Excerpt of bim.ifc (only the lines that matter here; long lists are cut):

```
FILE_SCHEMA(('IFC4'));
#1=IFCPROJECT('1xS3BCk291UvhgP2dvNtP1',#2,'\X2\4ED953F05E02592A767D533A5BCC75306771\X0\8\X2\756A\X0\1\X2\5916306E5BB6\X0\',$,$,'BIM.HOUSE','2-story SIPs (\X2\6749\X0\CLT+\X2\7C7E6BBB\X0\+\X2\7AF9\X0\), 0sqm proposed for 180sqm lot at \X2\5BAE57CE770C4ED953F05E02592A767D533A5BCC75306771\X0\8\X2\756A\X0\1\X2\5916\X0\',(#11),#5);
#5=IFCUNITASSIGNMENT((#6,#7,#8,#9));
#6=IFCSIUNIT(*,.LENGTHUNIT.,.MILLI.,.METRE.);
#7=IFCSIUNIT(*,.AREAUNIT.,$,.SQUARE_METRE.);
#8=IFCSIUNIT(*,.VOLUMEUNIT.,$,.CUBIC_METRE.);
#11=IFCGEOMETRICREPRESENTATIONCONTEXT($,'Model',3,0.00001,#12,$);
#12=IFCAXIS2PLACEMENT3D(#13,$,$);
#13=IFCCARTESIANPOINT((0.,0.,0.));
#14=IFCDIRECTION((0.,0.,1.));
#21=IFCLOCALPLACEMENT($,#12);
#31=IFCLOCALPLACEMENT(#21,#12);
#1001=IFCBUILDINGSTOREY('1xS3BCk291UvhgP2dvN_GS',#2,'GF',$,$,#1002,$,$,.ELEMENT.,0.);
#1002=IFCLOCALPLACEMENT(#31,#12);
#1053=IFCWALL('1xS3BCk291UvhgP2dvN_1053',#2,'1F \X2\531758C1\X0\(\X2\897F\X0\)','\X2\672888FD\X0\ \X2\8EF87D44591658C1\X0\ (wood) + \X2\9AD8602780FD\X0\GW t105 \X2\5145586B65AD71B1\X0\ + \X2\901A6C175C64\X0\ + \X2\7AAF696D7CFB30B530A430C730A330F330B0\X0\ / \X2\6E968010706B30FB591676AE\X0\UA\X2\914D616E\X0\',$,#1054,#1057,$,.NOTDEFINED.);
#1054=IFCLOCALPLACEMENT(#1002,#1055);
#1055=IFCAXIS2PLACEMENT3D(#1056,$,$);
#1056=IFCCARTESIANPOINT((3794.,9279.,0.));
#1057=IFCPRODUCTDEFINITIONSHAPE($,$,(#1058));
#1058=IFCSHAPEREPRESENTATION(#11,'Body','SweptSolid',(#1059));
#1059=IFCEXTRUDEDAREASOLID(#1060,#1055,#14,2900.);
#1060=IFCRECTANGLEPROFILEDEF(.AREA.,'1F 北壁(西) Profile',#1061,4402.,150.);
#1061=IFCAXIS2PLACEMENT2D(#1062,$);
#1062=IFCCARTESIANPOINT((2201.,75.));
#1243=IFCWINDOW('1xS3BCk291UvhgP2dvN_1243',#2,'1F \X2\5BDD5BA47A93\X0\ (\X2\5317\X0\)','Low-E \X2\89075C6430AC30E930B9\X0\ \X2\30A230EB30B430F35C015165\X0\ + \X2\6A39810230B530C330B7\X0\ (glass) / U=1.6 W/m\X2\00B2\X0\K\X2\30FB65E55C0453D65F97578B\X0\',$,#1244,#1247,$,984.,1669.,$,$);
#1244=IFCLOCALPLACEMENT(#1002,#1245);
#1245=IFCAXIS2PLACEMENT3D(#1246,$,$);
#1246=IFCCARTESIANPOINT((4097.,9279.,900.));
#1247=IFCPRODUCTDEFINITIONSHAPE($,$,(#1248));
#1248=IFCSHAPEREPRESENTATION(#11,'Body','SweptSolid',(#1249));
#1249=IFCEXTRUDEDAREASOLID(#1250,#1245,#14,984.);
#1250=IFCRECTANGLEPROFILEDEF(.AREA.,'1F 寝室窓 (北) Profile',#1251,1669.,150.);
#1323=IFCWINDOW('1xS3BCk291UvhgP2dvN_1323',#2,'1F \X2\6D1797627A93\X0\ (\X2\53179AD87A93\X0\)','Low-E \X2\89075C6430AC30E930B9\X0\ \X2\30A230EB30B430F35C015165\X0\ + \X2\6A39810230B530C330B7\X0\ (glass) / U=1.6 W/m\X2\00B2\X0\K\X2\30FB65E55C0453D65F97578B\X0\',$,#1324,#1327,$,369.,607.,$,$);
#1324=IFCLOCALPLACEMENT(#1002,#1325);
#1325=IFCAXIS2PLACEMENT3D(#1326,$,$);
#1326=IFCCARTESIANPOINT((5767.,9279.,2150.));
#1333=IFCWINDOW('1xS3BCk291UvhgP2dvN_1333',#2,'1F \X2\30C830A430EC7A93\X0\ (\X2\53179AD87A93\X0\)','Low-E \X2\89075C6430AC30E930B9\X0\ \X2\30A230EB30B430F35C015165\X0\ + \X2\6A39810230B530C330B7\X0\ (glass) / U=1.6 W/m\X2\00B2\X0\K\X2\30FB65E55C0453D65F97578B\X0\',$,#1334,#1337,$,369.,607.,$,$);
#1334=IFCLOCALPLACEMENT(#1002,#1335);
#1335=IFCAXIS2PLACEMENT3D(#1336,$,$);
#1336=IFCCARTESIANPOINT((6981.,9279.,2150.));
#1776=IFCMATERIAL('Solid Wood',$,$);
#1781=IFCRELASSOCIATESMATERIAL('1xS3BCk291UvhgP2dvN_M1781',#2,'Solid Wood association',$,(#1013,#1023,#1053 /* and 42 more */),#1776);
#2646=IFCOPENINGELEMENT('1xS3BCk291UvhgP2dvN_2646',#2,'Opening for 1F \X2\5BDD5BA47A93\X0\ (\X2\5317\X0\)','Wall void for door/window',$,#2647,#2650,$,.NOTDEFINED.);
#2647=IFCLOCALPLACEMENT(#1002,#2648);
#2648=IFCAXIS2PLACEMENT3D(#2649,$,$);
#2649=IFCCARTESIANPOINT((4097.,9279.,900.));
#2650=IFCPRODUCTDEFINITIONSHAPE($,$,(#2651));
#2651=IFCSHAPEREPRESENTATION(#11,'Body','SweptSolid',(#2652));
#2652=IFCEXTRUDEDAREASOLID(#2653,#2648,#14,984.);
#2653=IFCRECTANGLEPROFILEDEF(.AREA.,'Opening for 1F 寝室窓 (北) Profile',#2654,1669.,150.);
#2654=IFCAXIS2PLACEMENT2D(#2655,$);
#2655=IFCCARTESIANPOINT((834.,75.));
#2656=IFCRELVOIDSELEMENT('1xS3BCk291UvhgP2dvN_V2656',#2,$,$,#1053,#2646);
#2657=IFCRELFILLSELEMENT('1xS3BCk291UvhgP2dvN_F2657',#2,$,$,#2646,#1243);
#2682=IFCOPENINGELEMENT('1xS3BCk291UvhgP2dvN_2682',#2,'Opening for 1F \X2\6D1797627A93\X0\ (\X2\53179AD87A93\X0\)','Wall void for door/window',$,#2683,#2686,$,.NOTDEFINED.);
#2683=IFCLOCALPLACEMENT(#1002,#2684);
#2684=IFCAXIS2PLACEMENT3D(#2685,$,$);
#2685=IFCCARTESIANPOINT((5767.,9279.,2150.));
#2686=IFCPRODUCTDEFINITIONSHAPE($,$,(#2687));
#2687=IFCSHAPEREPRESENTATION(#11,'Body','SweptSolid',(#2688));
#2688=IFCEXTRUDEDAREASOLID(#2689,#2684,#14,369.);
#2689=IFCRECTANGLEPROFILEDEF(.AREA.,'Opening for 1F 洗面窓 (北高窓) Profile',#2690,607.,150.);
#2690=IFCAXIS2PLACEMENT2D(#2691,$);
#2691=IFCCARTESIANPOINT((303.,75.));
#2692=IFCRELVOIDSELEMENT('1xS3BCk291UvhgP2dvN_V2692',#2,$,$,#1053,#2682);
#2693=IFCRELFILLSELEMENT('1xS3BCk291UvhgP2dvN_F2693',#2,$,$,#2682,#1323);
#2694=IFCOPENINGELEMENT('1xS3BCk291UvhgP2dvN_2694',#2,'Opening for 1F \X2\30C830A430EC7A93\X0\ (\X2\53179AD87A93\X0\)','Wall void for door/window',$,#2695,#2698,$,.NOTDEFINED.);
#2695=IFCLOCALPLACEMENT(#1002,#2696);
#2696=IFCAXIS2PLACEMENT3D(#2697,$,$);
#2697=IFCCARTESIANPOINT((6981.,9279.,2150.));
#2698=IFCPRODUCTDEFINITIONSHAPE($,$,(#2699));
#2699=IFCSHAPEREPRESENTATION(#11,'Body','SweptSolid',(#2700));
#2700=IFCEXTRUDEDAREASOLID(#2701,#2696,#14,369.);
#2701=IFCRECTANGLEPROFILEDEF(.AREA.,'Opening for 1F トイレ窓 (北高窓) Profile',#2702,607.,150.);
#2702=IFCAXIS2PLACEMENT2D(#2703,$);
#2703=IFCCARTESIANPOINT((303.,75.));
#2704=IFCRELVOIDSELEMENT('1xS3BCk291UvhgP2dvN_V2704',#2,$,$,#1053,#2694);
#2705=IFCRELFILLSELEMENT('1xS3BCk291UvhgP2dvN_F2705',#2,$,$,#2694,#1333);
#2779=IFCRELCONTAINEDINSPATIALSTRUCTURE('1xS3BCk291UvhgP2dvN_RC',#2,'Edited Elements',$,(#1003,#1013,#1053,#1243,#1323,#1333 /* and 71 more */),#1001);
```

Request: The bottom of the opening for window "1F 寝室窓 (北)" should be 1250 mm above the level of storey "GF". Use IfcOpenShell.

```python
import numpy as np
import ifcopenshell
import ifcopenshell.api.geometry
import ifcopenshell.geom
import ifcopenshell.util.element
import ifcopenshell.util.placement
import ifcopenshell.util.shape
import ifcopenshell.util.unit

model = ifcopenshell.open("bim.ifc")
unit_scale = ifcopenshell.util.unit.calculate_unit_scale(model)

window = model.by_guid("1xS3BCk291UvhgP2dvN_1243")
opening = window.FillsVoids[0].RelatingOpeningElement
storey = ifcopenshell.util.element.get_container(window, ifc_class="IfcBuildingStorey")
level = ifcopenshell.util.placement.get_local_placement(storey.ObjectPlacement)[2, 3]

# The opening's origin need not be at the sill, so measure its lowest point.
shape = ifcopenshell.geom.create_shape(ifcopenshell.geom.settings(), opening)
bottom = ifcopenshell.util.shape.get_shape_bottom_elevation(shape, shape.geometry) / unit_scale
dz = level + 1250.0 - bottom

shift = np.array([0.0, 0.0, dz])
# The window is not placed relative to its opening, so move both.
for product in (opening, window):
    matrix = ifcopenshell.util.placement.get_local_placement(product.ObjectPlacement)
    matrix[:3, 3] += shift
    ifcopenshell.api.geometry.edit_object_placement(model, product=product, matrix=matrix, is_si=False)

print(f"moved by {dz * unit_scale:+.3f} m")

model.write("bim_rev.ifc")
```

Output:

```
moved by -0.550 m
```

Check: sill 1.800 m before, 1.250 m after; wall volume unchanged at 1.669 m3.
